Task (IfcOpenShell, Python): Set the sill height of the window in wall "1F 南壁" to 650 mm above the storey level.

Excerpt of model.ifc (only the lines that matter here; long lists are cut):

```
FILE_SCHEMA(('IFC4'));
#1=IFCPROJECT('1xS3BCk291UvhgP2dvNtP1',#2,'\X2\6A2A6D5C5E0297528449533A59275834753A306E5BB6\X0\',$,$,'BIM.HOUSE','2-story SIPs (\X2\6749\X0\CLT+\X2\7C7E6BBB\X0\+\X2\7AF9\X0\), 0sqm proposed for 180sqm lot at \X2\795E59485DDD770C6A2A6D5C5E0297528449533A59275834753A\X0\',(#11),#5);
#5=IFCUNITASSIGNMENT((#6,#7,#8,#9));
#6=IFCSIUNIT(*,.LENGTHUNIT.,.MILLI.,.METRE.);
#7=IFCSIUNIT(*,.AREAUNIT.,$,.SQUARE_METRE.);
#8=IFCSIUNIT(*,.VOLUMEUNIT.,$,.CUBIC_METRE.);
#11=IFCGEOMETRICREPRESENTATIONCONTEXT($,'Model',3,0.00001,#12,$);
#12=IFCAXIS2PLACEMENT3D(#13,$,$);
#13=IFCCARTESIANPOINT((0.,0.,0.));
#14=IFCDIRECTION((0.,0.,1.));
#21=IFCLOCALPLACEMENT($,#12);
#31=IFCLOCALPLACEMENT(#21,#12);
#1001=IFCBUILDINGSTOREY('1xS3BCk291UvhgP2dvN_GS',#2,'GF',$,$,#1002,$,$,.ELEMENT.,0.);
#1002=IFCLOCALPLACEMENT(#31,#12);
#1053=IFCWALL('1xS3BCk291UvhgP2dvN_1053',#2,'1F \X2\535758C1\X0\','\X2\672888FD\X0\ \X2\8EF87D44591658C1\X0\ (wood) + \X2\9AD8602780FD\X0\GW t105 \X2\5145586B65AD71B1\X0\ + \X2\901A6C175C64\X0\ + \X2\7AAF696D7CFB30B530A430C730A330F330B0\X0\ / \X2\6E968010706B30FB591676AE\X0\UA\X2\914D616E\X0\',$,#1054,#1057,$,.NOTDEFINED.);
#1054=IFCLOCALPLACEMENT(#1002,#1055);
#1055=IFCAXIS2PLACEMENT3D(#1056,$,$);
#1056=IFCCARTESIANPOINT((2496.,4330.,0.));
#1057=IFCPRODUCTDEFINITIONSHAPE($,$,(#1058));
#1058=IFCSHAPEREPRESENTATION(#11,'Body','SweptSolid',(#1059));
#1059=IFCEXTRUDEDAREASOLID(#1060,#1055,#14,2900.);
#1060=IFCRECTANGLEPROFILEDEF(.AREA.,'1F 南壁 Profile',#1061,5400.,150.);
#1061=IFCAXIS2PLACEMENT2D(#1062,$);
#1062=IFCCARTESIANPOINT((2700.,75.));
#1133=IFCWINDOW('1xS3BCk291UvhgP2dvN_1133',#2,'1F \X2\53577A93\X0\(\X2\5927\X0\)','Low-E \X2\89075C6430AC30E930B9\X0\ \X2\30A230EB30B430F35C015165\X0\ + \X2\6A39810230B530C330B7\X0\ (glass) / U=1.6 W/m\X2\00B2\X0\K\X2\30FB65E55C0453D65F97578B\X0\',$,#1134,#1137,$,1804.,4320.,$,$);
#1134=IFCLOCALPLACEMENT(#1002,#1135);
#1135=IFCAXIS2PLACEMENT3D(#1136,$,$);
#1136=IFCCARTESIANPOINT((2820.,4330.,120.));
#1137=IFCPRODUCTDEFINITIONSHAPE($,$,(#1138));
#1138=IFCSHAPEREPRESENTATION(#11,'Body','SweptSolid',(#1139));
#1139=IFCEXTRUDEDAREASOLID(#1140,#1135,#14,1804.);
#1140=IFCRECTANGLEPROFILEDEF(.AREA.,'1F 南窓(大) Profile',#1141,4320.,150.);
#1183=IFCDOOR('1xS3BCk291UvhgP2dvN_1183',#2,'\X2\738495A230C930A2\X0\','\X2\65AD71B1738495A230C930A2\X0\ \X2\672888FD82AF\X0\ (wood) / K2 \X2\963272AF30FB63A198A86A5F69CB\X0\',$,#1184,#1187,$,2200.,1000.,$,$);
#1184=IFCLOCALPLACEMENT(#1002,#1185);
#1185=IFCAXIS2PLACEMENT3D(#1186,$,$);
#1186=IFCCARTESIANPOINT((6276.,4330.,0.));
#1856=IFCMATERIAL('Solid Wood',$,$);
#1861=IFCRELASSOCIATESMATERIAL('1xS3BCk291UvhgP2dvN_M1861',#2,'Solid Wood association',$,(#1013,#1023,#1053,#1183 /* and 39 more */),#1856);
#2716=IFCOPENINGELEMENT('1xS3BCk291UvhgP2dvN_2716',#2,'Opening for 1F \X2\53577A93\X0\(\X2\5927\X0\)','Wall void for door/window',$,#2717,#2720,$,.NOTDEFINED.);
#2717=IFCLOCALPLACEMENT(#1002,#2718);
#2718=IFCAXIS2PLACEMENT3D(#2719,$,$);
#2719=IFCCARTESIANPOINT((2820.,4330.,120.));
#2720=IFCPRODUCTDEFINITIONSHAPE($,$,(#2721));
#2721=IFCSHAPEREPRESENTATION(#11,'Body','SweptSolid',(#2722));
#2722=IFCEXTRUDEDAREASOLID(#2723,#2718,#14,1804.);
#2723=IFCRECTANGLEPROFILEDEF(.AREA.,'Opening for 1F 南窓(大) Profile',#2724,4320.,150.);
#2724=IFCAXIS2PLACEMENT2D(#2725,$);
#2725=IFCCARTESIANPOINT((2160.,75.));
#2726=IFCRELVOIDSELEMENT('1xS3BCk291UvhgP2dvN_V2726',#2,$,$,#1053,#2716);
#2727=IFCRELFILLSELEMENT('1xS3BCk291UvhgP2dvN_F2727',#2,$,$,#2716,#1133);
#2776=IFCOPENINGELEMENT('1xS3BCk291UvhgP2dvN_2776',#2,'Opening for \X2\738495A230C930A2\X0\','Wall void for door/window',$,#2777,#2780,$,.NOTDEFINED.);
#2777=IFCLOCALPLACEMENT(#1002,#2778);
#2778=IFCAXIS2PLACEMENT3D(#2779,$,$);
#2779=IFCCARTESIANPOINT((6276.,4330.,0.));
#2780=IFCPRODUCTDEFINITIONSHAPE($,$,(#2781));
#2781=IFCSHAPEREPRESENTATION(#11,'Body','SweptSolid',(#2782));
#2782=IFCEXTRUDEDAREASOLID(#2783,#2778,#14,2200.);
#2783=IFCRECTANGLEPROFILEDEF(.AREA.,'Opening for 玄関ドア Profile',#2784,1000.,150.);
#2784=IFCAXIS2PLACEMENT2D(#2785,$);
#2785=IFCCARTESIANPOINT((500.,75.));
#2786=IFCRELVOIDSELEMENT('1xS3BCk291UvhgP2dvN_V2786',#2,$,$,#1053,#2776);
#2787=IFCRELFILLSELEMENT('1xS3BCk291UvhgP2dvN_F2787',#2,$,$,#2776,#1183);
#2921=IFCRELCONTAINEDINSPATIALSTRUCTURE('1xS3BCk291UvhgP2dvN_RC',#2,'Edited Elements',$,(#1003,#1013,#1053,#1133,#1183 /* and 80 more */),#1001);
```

```python
import numpy as np
import ifcopenshell
import ifcopenshell.api.geometry
import ifcopenshell.geom
import ifcopenshell.util.element
import ifcopenshell.util.placement
import ifcopenshell.util.shape
import ifcopenshell.util.unit

model = ifcopenshell.open("model.ifc")
unit_scale = ifcopenshell.util.unit.calculate_unit_scale(model)

window = model.by_id(1133)
opening = window.FillsVoids[0].RelatingOpeningElement
storey = ifcopenshell.util.element.get_container(window, ifc_class="IfcBuildingStorey")
level = ifcopenshell.util.placement.get_local_placement(storey.ObjectPlacement)[2, 3]

# The opening's origin need not be at the sill, so measure its lowest point.
shape = ifcopenshell.geom.create_shape(ifcopenshell.geom.settings(), opening)
bottom = ifcopenshell.util.shape.get_shape_bottom_elevation(shape, shape.geometry) / unit_scale
dz = level + 0.65 / unit_scale - bottom

shift = np.array([0.0, 0.0, dz])
# The window is not placed relative to its opening, so move both.
for product in (opening, window):
    matrix = ifcopenshell.util.placement.get_local_placement(product.ObjectPlacement)
    matrix[:3, 3] += shift
    ifcopenshell.api.geometry.edit_object_placement(model, product=product, matrix=matrix, is_si=False)

print(f"moved by {dz * unit_scale:+.3f} m")

model.write("model_updated.ifc")
```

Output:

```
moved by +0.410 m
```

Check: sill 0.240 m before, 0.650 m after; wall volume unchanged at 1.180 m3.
